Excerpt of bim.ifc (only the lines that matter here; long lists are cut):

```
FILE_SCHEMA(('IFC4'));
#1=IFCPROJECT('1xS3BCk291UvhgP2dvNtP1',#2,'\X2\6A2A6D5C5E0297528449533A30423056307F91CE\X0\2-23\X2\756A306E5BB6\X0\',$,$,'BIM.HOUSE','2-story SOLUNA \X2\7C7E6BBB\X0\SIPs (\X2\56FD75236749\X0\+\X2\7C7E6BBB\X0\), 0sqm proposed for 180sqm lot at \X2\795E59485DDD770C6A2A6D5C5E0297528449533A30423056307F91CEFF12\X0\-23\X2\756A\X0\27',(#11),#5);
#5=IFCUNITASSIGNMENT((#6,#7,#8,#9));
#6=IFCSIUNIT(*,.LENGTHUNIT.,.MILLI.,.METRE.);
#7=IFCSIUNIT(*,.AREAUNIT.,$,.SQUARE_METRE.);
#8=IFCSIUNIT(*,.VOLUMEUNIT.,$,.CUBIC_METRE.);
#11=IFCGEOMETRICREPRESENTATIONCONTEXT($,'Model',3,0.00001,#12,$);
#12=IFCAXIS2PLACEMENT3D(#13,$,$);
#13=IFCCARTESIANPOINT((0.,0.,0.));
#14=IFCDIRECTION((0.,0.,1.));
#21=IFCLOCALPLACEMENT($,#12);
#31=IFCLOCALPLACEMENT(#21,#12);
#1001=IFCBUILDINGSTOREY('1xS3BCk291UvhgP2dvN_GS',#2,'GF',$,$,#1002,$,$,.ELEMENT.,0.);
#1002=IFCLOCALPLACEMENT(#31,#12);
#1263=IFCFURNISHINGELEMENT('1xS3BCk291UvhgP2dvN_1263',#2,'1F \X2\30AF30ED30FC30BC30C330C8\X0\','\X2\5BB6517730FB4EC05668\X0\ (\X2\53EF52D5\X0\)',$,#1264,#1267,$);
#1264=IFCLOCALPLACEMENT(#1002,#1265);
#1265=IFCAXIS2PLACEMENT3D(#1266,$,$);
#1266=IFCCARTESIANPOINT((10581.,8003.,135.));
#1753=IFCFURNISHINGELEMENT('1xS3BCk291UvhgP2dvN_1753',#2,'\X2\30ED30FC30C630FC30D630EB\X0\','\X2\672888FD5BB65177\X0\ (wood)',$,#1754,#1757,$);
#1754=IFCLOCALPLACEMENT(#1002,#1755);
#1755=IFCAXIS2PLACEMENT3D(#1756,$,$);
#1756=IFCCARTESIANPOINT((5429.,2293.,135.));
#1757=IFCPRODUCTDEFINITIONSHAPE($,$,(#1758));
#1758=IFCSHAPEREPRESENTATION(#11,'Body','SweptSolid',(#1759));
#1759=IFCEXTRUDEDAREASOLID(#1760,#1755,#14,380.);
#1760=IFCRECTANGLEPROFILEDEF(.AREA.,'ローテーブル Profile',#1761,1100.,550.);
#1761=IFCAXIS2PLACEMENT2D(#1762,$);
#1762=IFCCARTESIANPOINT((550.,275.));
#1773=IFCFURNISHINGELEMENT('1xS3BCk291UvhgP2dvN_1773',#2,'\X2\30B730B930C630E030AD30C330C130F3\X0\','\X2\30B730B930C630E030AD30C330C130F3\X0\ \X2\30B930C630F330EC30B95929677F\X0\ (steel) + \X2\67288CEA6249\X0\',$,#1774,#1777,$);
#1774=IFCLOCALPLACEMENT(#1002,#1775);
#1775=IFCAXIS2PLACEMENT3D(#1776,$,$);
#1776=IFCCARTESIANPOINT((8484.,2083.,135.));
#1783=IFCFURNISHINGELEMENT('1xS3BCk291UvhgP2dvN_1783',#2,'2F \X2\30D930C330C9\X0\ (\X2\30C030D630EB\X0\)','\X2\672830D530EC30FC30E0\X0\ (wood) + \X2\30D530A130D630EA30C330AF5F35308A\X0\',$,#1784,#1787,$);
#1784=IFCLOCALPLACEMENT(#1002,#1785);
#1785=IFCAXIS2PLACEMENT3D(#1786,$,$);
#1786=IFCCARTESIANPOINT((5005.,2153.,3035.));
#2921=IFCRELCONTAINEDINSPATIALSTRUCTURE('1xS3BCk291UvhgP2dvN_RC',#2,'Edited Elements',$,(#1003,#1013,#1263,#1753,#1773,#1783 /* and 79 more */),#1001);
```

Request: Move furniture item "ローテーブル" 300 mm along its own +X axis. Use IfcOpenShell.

```python
import ifcopenshell
import ifcopenshell.api.geometry
import ifcopenshell.util.placement
import ifcopenshell.util.unit

model = ifcopenshell.open("bim.ifc")
unit_scale = ifcopenshell.util.unit.calculate_unit_scale(model)

item = model.by_guid("1xS3BCk291UvhgP2dvN_1753")
matrix = ifcopenshell.util.placement.get_local_placement(item.ObjectPlacement)
matrix[:3, 3] += matrix[:3, 0] * 0.3 / unit_scale
ifcopenshell.api.geometry.edit_object_placement(model, product=item, matrix=matrix, is_si=False)

print(ifcopenshell.util.placement.get_local_placement(item.ObjectPlacement).round(3) + 0.0)

model.write("bim_edited.ifc")
```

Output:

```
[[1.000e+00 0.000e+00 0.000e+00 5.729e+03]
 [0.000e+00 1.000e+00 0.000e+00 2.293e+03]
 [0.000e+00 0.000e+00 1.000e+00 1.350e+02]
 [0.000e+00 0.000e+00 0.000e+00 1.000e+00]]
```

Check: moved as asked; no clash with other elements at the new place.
